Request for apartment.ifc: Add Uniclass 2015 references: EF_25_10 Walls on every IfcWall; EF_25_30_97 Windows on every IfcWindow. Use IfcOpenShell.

First a look at what the model holds.

```python
import ifcopenshell

model = ifcopenshell.open("apartment.ifc")
print(model.schema)
print("classifications:", [c.Name for c in model.by_type("IfcClassification")])
for ifc_class in ("IfcDoor", "IfcRoof", "IfcStair", "IfcWall", "IfcWindow"):
    print(ifc_class, len(model.by_type(ifc_class)))
```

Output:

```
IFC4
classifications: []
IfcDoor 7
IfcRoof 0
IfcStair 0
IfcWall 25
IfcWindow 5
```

```python
import ifcopenshell
import ifcopenshell.api.classification

model = ifcopenshell.open("apartment.ifc")

system = ifcopenshell.api.classification.add_classification(model, classification="Uniclass 2015")

codes = {
    "IfcWall": ("EF_25_10", "Walls"),
    "IfcWindow": ("EF_25_30_97", "Windows"),
}
for ifc_class, (code, name) in codes.items():
    products = model.by_type(ifc_class)
    ifcopenshell.api.classification.add_reference(
        model, products=products, classification=system, identification=code, name=name
    )
    print(code, len(products))

model.write("apartment_edited.ifc")
```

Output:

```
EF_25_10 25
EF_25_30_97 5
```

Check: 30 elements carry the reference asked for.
